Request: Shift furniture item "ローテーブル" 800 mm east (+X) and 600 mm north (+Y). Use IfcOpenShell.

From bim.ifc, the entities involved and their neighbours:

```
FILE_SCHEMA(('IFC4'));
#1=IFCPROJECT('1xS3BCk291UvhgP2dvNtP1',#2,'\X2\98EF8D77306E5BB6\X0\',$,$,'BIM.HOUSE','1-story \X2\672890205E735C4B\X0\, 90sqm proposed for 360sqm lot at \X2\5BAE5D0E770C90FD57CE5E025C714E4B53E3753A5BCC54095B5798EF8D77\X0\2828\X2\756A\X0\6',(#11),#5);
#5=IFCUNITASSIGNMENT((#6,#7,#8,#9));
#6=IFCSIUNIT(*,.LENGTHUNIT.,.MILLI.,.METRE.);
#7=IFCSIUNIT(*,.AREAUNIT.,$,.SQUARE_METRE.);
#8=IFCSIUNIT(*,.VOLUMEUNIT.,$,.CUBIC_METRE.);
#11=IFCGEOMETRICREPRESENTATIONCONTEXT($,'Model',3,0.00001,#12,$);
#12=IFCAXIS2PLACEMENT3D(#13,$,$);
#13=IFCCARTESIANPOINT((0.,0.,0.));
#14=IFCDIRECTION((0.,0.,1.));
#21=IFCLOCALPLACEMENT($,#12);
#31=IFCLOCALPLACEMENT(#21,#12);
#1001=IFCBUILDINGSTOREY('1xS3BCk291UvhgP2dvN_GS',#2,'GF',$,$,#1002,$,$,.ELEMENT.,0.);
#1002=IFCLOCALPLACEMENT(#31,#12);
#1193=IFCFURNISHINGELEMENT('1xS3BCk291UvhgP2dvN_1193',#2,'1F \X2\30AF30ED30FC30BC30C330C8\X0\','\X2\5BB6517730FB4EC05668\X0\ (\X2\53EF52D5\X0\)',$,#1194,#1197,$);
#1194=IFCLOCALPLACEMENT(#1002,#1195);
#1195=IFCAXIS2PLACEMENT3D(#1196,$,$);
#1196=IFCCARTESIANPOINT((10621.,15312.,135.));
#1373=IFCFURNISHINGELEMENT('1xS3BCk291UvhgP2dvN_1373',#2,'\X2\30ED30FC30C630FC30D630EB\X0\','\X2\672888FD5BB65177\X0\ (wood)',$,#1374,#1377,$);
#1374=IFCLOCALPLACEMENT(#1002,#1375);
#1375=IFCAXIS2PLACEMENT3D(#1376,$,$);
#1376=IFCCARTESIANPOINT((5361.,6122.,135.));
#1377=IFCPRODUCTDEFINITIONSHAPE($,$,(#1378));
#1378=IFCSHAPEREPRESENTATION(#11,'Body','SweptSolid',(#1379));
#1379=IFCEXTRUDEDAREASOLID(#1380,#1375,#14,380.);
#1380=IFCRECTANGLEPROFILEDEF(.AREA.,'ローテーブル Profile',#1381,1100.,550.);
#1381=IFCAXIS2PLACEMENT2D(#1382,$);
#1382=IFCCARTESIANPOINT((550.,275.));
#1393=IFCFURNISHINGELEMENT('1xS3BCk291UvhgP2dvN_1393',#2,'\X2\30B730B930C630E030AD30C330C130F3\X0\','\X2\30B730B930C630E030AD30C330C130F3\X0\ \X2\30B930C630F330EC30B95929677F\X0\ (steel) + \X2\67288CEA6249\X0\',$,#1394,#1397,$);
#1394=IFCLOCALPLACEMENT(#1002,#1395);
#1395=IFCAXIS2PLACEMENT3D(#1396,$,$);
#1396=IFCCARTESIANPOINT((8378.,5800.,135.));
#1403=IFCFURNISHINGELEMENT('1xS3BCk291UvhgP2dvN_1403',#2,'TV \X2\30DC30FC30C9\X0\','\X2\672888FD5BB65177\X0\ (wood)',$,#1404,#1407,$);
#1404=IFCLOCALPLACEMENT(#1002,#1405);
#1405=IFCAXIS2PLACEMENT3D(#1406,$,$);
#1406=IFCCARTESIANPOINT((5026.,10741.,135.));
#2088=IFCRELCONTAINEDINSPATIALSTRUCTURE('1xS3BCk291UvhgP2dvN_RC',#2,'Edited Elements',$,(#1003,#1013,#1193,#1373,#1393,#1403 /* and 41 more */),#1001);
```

```python
import ifcopenshell
import ifcopenshell.api.geometry
import ifcopenshell.util.placement

model = ifcopenshell.open("bim.ifc")

item = model.by_guid("1xS3BCk291UvhgP2dvN_1373")
matrix = ifcopenshell.util.placement.get_local_placement(item.ObjectPlacement)
matrix[0, 3] += 800.0
matrix[1, 3] += 600.0
ifcopenshell.api.geometry.edit_object_placement(model, product=item, matrix=matrix, is_si=False)

print(ifcopenshell.util.placement.get_local_placement(item.ObjectPlacement).round(3) + 0.0)

model.write("bim_updated.ifc")
```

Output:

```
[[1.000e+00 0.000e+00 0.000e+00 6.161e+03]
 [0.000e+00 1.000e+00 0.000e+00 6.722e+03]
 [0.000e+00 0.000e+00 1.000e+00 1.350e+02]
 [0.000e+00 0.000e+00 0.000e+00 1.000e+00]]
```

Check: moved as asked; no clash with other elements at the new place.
